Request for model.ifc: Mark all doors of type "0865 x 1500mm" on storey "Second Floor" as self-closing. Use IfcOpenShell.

First a look at what the model holds.

```python
import ifcopenshell
import ifcopenshell.util.element

model = ifcopenshell.open("model.ifc")
print(model.schema)
storey = next(s for s in model.by_type("IfcBuildingStorey") if s.Name == "Second Floor")
doors = [e for e in ifcopenshell.util.element.get_decomposition(storey) if e.is_a("IfcDoor")]
seen = {}
for e in doors:
    element_type = ifcopenshell.util.element.get_type(e)
    key = (element_type.Name if element_type != e and element_type else None, ifcopenshell.util.element.get_pset(e, "Pset_DoorCommon", "SelfClosing"))
    seen[key] = seen.get(key, 0) + 1
for (name, value), count in sorted(seen.items(), key=str):
    print(count, "x", name, "|", value)
```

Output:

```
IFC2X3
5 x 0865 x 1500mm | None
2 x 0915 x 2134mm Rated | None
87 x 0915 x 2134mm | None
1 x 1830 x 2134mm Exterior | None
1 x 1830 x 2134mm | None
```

```python
import ifcopenshell
import ifcopenshell.api.pset
import ifcopenshell.util.element

model = ifcopenshell.open("model.ifc")

storey = next(s for s in model.by_type("IfcBuildingStorey") if s.Name == "Second Floor")
doors = [e for e in ifcopenshell.util.element.get_decomposition(storey) if e.is_a("IfcDoor")]

count = 0
for e in doors:
    element_type = ifcopenshell.util.element.get_type(e)
    if element_type in (None, e) or element_type.Name != "0865 x 1500mm":
        continue
    # add_pset returns the element's existing set when there is one.
    pset = ifcopenshell.api.pset.add_pset(model, product=e, name="Pset_DoorCommon")
    ifcopenshell.api.pset.edit_pset(model, pset=pset, properties={"SelfClosing": True})
    count += 1

print(count, "doors updated")

model.write("model_v2.ifc")
```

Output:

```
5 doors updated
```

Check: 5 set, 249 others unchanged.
